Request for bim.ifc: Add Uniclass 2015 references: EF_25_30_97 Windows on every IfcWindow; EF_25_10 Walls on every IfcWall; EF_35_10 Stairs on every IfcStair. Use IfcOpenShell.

First a look at what the model holds.

```python
import ifcopenshell

model = ifcopenshell.open("bim.ifc")
print(model.schema)
print("classifications:", [c.Name for c in model.by_type("IfcClassification")])
for ifc_class in ("IfcDoor", "IfcRoof", "IfcStair", "IfcWall", "IfcWindow"):
    print(ifc_class, len(model.by_type(ifc_class)))
```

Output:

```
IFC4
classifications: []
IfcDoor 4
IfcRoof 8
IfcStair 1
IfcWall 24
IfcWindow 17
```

```python
import ifcopenshell
import ifcopenshell.api.classification

model = ifcopenshell.open("bim.ifc")

system = ifcopenshell.api.classification.add_classification(model, classification="Uniclass 2015")

codes = {
    "IfcWindow": ("EF_25_30_97", "Windows"),
    "IfcWall": ("EF_25_10", "Walls"),
    "IfcStair": ("EF_35_10", "Stairs"),
}
for ifc_class, (code, name) in codes.items():
    products = model.by_type(ifc_class)
    ifcopenshell.api.classification.add_reference(
        model, products=products, classification=system, identification=code, name=name
    )
    print(code, len(products))

model.write("bim-out.ifc")
```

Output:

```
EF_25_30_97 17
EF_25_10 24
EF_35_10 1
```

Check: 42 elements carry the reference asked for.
